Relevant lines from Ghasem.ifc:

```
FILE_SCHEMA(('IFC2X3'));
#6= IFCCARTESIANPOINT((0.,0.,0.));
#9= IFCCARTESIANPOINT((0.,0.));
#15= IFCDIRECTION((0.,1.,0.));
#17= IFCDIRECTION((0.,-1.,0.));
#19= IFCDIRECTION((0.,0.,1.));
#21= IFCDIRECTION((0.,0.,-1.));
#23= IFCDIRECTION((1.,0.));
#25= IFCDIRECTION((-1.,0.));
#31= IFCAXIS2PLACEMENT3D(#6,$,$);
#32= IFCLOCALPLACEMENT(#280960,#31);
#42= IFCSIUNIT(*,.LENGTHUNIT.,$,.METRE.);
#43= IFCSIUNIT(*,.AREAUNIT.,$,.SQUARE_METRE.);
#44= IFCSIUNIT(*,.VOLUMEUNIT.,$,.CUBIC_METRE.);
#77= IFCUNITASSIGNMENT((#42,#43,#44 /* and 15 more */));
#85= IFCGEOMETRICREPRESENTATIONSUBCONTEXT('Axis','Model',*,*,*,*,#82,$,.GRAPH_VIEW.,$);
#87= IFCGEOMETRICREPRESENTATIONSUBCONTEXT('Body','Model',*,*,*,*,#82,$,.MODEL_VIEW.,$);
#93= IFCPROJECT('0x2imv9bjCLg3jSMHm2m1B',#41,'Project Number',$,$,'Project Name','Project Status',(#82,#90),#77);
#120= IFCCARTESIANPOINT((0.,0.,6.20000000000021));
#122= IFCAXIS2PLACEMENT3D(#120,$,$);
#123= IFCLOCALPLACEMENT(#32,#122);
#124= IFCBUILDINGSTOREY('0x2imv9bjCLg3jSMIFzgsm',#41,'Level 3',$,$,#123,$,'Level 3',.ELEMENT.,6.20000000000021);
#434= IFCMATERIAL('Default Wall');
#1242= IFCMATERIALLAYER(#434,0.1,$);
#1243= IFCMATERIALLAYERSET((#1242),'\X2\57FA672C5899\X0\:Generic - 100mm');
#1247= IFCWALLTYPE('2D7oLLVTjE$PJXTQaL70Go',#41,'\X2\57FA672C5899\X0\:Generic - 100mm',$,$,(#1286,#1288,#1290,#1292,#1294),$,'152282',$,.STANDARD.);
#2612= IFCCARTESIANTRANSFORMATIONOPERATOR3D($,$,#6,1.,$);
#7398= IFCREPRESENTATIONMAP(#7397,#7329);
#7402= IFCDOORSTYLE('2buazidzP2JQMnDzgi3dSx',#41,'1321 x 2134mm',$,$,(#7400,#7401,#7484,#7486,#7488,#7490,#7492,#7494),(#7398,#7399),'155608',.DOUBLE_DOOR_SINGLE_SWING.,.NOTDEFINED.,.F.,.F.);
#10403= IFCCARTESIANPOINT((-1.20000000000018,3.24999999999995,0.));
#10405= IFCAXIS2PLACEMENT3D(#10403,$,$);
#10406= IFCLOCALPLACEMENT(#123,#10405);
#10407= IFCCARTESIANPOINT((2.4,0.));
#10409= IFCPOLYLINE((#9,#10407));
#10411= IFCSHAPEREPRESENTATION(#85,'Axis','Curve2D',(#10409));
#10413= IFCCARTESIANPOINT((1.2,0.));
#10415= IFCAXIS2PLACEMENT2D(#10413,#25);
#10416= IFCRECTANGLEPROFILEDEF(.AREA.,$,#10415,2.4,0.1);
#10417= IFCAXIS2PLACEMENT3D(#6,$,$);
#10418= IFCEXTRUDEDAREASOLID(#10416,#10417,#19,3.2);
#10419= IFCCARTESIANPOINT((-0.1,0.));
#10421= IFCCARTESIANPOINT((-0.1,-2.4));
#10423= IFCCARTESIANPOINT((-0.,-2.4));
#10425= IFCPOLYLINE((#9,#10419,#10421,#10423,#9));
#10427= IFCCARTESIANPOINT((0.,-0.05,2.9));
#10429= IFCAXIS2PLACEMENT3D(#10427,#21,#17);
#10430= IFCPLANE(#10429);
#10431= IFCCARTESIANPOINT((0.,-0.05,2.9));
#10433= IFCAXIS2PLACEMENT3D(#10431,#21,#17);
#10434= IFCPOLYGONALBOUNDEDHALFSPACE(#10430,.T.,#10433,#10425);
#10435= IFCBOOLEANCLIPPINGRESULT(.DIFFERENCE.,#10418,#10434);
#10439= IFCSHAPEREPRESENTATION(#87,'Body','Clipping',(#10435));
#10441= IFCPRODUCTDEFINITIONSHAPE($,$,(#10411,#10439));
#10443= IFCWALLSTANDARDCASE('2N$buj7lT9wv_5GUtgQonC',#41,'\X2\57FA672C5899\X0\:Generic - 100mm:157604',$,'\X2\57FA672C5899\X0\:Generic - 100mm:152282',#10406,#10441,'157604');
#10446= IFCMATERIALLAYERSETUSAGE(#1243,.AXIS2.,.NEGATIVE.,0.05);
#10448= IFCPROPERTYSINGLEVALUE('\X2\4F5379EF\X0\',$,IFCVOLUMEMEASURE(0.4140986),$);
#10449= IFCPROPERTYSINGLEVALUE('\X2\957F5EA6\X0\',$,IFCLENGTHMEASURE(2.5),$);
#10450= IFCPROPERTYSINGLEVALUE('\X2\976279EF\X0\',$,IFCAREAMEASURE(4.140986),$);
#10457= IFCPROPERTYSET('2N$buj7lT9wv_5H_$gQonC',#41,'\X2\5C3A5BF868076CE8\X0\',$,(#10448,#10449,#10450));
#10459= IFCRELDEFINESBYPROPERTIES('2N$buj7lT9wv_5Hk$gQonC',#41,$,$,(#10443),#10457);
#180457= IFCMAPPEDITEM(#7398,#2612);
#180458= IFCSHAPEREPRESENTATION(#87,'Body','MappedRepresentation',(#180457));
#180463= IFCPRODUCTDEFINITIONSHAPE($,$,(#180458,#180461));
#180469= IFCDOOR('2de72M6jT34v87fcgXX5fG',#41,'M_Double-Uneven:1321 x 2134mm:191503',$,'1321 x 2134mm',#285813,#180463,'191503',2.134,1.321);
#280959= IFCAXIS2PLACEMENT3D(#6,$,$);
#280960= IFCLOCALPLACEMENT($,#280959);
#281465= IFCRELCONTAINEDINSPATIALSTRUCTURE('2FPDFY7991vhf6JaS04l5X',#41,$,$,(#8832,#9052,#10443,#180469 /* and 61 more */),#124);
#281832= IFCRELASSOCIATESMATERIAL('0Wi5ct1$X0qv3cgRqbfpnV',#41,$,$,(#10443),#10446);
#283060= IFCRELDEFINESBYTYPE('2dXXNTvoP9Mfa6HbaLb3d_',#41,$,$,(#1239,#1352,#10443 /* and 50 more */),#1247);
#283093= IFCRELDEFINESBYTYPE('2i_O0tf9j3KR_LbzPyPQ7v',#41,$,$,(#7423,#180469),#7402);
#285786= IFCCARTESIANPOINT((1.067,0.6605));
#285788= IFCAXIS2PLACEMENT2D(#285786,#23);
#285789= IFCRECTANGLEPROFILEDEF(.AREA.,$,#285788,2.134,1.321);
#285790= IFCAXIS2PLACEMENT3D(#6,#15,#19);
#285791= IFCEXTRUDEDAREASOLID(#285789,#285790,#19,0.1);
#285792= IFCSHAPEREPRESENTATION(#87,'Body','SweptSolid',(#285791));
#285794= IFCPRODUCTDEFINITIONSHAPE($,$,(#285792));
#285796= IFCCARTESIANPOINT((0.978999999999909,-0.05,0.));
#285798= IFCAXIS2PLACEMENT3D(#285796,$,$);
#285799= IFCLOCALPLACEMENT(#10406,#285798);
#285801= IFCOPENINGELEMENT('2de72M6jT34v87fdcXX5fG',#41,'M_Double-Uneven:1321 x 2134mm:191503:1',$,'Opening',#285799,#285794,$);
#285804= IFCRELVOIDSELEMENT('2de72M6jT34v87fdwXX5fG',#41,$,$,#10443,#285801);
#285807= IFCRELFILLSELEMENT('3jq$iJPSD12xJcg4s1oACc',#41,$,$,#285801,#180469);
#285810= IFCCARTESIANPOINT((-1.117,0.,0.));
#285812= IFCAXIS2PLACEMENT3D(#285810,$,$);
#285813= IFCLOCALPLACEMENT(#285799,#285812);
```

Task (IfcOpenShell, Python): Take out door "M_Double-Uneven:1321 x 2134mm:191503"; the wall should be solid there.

```python
import ifcopenshell
import ifcopenshell.api.feature
import ifcopenshell.api.pset
import ifcopenshell.api.root
import ifcopenshell.geom
import ifcopenshell.util.element
import ifcopenshell.util.shape
import ifcopenshell.util.unit

model = ifcopenshell.open("Ghasem.ifc")
area_scale = ifcopenshell.util.unit.calculate_unit_scale(model, "AREAUNIT")
volume_scale = ifcopenshell.util.unit.calculate_unit_scale(model, "VOLUMEUNIT")
settings = ifcopenshell.geom.settings()


def volume(element):
    """Net volume in cubic metres, openings subtracted."""
    shape = ifcopenshell.geom.create_shape(settings, element)
    return ifcopenshell.util.shape.get_volume(shape.geometry)


door = model.by_guid("2de72M6jT34v87fcgXX5fG")
opening = door.FillsVoids[0].RelatingOpeningElement
wall = opening.VoidsElements[0].RelatingBuildingElement
before = volume(wall)

ifcopenshell.api.root.remove_product(model, product=door)
ifcopenshell.api.feature.remove_feature(model, feature=opening)

after = volume(wall)
thickness = 0.1  # wall thickness in metres

# Update the wall's stored quantities.
pset = model.by_id(ifcopenshell.util.element.get_pset(wall, "尺寸标注", should_inherit=False)["id"])
ifcopenshell.api.pset.edit_pset(model, pset=pset, properties={
    "体积": model.create_entity("IfcVolumeMeasure", after / volume_scale),
    "面积": model.create_entity("IfcAreaMeasure", after / thickness / area_scale),
})

print(f"wall volume {before:.3f} -> {after:.3f} m3")

model.write("Ghasem_updated.ifc")
```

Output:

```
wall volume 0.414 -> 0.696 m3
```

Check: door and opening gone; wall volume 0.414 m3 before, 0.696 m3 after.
